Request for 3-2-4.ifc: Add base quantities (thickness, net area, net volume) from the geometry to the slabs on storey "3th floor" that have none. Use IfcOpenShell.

First a look at what the model holds.

```python
import ifcopenshell
import ifcopenshell.util.element
import ifcopenshell.util.unit

model = ifcopenshell.open("3-2-4.ifc")
print(model.schema)
for unit_type in ("LENGTHUNIT", "AREAUNIT", "VOLUMEUNIT"):
    print(unit_type, ifcopenshell.util.unit.calculate_unit_scale(model, unit_type))
storey = next(s for s in model.by_type("IfcBuildingStorey") if s.Name == "3th floor")
slabs = [e for e in ifcopenshell.util.element.get_decomposition(storey) if e.is_a("IfcSlab")]
for e in sorted(slabs, key=lambda e: e.id()):
    print(e.id(), e.is_a(), e.Name, list(ifcopenshell.util.element.get_psets(e, qtos_only=True)), sep=" | ")
```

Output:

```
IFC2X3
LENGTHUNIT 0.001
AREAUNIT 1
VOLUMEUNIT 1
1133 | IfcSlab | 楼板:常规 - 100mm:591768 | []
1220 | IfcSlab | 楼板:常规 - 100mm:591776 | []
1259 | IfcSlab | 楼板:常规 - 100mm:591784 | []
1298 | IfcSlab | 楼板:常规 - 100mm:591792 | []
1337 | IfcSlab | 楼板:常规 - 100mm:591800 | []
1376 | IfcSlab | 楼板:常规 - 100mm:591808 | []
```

```python
import ifcopenshell
import ifcopenshell.api.pset
import ifcopenshell.geom
import ifcopenshell.util.element
import ifcopenshell.util.shape
import ifcopenshell.util.unit

model = ifcopenshell.open("3-2-4.ifc")
unit_scale = ifcopenshell.util.unit.calculate_unit_scale(model)
area_scale = ifcopenshell.util.unit.calculate_unit_scale(model, "AREAUNIT")
volume_scale = ifcopenshell.util.unit.calculate_unit_scale(model, "VOLUMEUNIT")
settings = ifcopenshell.geom.settings()

storey = next(s for s in model.by_type("IfcBuildingStorey") if s.Name == "3th floor")
slabs = [e for e in ifcopenshell.util.element.get_decomposition(storey) if e.is_a("IfcSlab")]

for e in sorted(slabs, key=lambda e: e.id()):
    if ifcopenshell.util.element.get_psets(e, qtos_only=True, should_inherit=False):
        continue
    # Geometry comes back in metres, in the element's own axes.
    shape = ifcopenshell.geom.create_shape(settings, e)
    values = {
        "Width": ifcopenshell.util.shape.get_z(shape.geometry) / unit_scale,
        "NetArea": ifcopenshell.util.shape.get_footprint_area(shape.geometry) / area_scale,
        "NetVolume": ifcopenshell.util.shape.get_volume(shape.geometry) / volume_scale,
    }
    qto = ifcopenshell.api.pset.add_qto(model, product=e, name="BaseQuantities")
    ifcopenshell.api.pset.edit_qto(model, qto=qto, properties=values)
    print(e.id(), {k: round(v, 3) for k, v in values.items()})

model.write("3-2-4_updated.ifc")
```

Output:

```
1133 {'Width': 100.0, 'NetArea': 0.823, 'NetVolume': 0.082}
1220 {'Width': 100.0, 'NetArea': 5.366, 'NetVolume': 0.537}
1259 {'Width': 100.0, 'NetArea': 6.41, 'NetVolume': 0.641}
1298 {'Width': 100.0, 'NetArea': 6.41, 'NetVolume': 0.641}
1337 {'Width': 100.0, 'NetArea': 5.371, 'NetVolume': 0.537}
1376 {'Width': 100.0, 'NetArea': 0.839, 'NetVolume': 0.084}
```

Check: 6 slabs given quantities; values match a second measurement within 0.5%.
